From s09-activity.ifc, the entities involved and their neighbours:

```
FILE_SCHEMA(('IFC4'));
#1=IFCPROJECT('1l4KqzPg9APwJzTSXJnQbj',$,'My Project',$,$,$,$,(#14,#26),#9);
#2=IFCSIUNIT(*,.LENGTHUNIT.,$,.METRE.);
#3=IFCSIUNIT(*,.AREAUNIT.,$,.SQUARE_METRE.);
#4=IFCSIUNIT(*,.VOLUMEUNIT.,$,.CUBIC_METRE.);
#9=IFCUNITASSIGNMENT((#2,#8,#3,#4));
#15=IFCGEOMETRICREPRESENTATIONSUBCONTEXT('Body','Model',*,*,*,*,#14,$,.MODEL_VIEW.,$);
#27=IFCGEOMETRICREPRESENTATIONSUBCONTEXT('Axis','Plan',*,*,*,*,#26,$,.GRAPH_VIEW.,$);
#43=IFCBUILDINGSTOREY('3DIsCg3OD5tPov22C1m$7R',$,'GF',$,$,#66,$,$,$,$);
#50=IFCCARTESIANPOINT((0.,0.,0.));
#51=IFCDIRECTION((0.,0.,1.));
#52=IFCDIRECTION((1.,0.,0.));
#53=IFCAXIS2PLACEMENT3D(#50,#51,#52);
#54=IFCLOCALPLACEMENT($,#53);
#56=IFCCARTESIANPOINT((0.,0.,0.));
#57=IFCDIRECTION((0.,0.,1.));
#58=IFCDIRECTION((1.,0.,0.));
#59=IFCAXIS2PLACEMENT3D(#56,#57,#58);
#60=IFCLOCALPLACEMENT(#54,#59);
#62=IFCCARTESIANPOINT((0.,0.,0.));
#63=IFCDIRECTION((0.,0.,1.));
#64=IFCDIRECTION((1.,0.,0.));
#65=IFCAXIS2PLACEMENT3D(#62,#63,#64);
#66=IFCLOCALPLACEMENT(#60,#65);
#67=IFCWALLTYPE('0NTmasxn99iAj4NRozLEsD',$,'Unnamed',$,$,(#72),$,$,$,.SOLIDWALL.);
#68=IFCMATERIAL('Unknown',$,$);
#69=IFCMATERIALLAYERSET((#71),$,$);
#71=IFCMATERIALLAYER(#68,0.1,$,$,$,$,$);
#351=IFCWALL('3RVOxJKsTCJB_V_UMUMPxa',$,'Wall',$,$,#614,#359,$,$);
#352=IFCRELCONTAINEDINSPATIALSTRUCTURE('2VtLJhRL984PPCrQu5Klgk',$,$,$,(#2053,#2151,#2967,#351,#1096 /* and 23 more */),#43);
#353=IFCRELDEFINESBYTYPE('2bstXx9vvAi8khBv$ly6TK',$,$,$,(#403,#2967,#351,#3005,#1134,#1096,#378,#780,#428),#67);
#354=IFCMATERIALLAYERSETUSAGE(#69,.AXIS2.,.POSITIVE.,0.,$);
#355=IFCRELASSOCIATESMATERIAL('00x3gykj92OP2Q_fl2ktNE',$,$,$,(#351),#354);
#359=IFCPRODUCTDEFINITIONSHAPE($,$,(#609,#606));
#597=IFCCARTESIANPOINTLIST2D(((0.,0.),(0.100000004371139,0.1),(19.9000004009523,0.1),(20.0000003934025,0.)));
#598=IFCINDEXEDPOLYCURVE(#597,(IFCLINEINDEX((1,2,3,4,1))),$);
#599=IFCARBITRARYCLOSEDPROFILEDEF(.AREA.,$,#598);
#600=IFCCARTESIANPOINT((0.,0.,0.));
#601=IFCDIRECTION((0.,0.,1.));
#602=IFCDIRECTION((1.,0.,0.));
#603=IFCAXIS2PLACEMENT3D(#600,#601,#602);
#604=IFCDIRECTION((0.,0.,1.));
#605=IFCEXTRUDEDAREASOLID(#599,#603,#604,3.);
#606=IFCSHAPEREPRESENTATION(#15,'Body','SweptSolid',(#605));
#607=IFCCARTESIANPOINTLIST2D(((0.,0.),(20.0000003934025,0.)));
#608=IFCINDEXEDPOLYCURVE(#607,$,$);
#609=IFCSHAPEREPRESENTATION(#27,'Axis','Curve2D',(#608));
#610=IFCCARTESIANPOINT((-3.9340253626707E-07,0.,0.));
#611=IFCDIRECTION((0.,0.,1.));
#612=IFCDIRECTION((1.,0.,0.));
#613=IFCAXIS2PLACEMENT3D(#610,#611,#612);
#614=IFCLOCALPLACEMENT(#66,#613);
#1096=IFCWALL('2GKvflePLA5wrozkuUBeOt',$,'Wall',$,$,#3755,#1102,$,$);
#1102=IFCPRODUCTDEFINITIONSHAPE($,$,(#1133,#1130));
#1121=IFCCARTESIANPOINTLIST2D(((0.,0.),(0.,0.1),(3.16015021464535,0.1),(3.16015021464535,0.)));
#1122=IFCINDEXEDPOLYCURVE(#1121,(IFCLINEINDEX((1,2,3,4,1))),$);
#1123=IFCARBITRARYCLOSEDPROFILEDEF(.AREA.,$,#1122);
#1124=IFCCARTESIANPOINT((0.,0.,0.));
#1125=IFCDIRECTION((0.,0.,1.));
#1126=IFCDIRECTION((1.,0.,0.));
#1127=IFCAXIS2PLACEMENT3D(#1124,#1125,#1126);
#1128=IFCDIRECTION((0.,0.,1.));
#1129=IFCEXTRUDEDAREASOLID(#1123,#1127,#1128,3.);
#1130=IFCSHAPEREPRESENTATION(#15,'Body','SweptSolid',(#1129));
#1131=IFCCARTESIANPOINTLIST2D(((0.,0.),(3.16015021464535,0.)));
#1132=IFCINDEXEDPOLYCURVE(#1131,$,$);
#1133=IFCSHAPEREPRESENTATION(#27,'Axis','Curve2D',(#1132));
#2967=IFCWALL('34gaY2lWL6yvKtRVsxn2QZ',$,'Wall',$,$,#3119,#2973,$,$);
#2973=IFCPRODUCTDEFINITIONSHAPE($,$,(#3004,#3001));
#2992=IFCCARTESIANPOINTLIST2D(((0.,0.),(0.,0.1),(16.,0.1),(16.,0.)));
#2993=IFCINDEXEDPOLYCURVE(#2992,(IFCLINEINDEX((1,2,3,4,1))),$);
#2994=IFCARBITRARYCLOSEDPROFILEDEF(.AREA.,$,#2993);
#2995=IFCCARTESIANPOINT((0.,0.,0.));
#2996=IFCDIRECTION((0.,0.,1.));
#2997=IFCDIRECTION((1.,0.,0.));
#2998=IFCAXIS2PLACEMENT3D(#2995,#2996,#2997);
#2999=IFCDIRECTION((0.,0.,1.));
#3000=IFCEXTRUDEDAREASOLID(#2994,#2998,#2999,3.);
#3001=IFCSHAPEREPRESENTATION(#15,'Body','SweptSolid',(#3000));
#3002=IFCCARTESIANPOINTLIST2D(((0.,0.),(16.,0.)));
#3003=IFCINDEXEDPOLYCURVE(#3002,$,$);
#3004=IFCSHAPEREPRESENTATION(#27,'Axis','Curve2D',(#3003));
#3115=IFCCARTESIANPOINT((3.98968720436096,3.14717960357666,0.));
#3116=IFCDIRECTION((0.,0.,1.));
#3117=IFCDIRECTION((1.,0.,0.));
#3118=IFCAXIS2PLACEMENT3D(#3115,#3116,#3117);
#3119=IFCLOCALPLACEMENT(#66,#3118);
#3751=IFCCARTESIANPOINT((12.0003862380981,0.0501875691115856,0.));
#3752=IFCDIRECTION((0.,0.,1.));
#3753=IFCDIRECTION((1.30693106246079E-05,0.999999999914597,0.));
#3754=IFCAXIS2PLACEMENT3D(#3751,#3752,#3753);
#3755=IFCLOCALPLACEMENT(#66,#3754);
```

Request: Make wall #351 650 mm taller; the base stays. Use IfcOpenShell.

```python
import ifcopenshell
import ifcopenshell.geom
import ifcopenshell.util.representation
import ifcopenshell.util.shape

model = ifcopenshell.open("s09-activity.ifc")
settings = ifcopenshell.geom.settings()


def volume(element):
    """Net volume in cubic metres, openings subtracted."""
    shape = ifcopenshell.geom.create_shape(settings, element)
    return ifcopenshell.util.shape.get_volume(shape.geometry)


wall = model.by_guid("3RVOxJKsTCJB_V_UMUMPxa")
before = volume(wall)

body = ifcopenshell.util.representation.get_representation(wall, "Model", "Body")
solid = body.Items[0]
old_height = solid.Depth
solid.Depth += 0.65
after = volume(wall)

print(f"height {old_height:g} -> {solid.Depth:g}, volume {before:.3f} -> {after:.3f} m3")

model.write("s09-activity_rev.ifc")
```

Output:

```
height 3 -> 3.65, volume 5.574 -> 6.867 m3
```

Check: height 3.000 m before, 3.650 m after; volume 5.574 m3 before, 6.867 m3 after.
